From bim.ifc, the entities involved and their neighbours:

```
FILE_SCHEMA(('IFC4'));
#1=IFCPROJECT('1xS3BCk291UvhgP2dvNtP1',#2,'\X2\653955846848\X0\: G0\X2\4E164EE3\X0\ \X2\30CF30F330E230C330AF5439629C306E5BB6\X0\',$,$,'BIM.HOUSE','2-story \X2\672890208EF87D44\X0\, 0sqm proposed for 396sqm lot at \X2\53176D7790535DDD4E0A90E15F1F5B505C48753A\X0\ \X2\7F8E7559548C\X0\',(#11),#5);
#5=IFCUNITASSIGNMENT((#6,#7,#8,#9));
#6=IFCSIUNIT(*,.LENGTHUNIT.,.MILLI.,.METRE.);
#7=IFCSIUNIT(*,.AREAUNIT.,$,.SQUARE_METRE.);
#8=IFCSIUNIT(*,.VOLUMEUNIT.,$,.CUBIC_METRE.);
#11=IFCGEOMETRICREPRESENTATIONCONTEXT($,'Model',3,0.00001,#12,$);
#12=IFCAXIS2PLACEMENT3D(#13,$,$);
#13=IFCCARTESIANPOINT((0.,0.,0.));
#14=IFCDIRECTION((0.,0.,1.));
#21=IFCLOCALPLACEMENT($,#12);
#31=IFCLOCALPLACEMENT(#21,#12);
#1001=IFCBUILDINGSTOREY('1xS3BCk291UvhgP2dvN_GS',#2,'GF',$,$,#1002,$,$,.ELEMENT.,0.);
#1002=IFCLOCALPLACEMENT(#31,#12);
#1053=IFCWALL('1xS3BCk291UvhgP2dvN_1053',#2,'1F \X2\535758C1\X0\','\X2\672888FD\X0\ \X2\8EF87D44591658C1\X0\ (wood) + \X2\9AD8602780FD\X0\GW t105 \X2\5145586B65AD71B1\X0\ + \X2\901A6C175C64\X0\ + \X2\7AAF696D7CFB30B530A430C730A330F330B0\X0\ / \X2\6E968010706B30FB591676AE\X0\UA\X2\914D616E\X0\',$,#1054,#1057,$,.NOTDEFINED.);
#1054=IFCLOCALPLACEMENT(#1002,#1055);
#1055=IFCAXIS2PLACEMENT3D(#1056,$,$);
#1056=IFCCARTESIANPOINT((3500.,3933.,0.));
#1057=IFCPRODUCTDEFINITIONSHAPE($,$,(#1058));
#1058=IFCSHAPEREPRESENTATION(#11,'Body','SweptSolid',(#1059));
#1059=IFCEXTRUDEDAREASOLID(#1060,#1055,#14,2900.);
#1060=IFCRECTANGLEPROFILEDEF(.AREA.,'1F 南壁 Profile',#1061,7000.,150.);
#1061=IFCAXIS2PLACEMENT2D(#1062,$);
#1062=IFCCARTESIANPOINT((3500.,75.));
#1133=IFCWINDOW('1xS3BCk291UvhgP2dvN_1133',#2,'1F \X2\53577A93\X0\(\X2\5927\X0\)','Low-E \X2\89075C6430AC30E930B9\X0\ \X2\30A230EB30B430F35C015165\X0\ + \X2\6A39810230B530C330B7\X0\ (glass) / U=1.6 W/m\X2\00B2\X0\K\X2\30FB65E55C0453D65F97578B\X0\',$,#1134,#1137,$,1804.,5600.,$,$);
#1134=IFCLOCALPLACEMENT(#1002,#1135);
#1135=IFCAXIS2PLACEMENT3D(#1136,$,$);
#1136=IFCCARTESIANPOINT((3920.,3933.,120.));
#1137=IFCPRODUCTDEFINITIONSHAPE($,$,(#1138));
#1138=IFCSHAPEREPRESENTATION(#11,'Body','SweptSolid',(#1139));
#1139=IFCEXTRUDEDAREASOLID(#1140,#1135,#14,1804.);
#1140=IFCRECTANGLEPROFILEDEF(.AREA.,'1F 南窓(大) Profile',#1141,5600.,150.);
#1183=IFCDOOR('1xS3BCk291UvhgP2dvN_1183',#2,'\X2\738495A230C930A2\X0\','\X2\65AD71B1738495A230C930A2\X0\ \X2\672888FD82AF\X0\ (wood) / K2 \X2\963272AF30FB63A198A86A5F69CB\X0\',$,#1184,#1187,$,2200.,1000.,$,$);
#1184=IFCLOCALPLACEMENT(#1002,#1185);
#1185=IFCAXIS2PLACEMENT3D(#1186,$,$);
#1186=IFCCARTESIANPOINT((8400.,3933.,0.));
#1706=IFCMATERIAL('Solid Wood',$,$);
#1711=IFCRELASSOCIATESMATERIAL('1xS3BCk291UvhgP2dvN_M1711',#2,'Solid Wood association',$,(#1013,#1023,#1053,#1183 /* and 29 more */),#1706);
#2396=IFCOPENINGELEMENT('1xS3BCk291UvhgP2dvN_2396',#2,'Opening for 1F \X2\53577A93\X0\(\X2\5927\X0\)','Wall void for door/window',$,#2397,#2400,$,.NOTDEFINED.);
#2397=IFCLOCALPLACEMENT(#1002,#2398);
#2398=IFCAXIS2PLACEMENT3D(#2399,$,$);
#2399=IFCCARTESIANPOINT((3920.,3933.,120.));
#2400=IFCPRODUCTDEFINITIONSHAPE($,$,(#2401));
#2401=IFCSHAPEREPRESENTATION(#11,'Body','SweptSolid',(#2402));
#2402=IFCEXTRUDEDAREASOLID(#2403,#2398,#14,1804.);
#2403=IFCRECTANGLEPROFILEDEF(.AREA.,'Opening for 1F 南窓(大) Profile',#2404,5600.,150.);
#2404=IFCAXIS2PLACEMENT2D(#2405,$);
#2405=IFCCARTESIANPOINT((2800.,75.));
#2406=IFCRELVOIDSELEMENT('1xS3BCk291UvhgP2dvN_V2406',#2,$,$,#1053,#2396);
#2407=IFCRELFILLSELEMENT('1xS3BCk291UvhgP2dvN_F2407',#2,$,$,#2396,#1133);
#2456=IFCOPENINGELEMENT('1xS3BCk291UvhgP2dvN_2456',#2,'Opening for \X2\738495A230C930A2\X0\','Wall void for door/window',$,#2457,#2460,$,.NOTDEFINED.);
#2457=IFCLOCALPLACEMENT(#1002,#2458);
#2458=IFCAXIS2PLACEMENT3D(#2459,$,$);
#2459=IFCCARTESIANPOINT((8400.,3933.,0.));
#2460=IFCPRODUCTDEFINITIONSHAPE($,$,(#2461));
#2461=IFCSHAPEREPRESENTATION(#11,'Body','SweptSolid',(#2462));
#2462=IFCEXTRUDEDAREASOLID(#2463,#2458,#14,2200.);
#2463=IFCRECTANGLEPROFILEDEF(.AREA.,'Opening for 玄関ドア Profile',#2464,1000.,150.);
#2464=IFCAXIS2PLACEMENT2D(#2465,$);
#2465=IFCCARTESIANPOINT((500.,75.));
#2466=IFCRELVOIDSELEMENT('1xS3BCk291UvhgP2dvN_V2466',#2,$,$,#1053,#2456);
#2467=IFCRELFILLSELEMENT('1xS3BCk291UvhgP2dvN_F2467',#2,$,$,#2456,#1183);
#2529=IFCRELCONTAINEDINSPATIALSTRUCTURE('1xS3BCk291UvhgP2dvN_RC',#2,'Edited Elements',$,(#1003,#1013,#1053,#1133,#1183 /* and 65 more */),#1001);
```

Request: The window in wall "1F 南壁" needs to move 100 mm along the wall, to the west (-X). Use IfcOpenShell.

```python
import ifcopenshell
import ifcopenshell.api.geometry
import ifcopenshell.util.placement
import ifcopenshell.util.unit

model = ifcopenshell.open("bim.ifc")
unit_scale = ifcopenshell.util.unit.calculate_unit_scale(model)

window = model.by_id(1133)
opening = window.FillsVoids[0].RelatingOpeningElement
wall = opening.VoidsElements[0].RelatingBuildingElement

wall_matrix = ifcopenshell.util.placement.get_local_placement(wall.ObjectPlacement)
shift = wall_matrix[:3, 0] * -0.1 / unit_scale
before = ifcopenshell.util.placement.get_local_placement(window.ObjectPlacement)[:3, 3].copy()

# The window is not placed relative to its opening, so move both.
for product in (opening, window):
    matrix = ifcopenshell.util.placement.get_local_placement(product.ObjectPlacement)
    matrix[:3, 3] += shift
    ifcopenshell.api.geometry.edit_object_placement(model, product=product, matrix=matrix, is_si=False)

after = ifcopenshell.util.placement.get_local_placement(window.ObjectPlacement)[:3, 3]
print("window moved by", (after - before).round(3) + 0.0)

model.write("bim_edited.ifc")
```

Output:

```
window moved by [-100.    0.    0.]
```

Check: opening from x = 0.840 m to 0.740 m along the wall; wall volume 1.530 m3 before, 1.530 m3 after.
